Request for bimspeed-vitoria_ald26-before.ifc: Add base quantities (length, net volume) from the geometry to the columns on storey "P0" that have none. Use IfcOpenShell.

First a look at what the model holds.

```python
import ifcopenshell
import ifcopenshell.util.element
import ifcopenshell.util.unit

model = ifcopenshell.open("bimspeed-vitoria_ald26-before.ifc")
print(model.schema)
for unit_type in ("LENGTHUNIT", "AREAUNIT", "VOLUMEUNIT"):
    print(unit_type, ifcopenshell.util.unit.calculate_unit_scale(model, unit_type))
storey = next(s for s in model.by_type("IfcBuildingStorey") if s.Name == "P0")
columns = [e for e in ifcopenshell.util.element.get_decomposition(storey) if e.is_a("IfcColumn")]
for e in sorted(columns, key=lambda e: e.id()):
    print(e.id(), e.is_a(), e.Name, list(ifcopenshell.util.element.get_psets(e, qtos_only=True)), sep=" | ")
```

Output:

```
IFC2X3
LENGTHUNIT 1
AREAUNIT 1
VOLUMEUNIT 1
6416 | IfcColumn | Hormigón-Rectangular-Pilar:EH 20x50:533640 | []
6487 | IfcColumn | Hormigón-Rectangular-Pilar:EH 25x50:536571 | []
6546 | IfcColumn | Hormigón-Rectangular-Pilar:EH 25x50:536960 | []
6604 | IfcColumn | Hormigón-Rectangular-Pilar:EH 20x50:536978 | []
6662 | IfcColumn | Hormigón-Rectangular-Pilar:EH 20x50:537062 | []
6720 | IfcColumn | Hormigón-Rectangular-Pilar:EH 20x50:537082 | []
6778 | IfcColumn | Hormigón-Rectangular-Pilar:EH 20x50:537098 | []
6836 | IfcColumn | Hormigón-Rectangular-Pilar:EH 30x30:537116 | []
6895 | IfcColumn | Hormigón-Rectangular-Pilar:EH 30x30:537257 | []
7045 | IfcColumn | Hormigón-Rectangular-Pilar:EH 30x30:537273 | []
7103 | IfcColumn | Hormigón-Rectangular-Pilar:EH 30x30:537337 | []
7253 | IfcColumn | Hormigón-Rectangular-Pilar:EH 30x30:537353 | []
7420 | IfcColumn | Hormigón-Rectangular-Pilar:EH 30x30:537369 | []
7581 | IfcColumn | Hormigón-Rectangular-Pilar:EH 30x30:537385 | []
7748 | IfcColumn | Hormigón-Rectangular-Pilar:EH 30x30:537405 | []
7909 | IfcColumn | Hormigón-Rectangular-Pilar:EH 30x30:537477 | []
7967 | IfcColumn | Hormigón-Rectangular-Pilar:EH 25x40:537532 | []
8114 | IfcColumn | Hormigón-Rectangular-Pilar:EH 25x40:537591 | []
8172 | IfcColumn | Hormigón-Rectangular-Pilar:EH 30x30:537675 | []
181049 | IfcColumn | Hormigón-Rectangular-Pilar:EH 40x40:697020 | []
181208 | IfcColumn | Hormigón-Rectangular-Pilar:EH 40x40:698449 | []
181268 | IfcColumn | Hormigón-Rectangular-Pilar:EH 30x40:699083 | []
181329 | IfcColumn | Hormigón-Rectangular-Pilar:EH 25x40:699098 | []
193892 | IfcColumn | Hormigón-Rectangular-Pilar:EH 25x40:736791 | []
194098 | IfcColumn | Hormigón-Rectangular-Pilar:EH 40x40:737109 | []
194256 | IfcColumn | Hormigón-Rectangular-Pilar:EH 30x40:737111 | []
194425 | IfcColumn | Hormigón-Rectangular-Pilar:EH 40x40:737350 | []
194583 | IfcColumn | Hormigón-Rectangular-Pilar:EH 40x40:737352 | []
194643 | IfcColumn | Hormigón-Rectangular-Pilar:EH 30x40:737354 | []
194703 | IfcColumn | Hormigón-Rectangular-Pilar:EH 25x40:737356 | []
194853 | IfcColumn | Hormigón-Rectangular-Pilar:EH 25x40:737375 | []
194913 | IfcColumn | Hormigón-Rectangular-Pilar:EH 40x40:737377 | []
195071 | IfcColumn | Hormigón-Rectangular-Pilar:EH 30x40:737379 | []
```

```python
import ifcopenshell
import ifcopenshell.api.pset
import ifcopenshell.geom
import ifcopenshell.util.element
import ifcopenshell.util.shape
import ifcopenshell.util.unit

model = ifcopenshell.open("bimspeed-vitoria_ald26-before.ifc")
unit_scale = ifcopenshell.util.unit.calculate_unit_scale(model)
volume_scale = ifcopenshell.util.unit.calculate_unit_scale(model, "VOLUMEUNIT")
settings = ifcopenshell.geom.settings()

storey = next(s for s in model.by_type("IfcBuildingStorey") if s.Name == "P0")
columns = [e for e in ifcopenshell.util.element.get_decomposition(storey) if e.is_a("IfcColumn")]

for e in sorted(columns, key=lambda e: e.id()):
    if ifcopenshell.util.element.get_psets(e, qtos_only=True, should_inherit=False):
        continue
    # Geometry comes back in metres, in the element's own axes.
    shape = ifcopenshell.geom.create_shape(settings, e)
    values = {
        "Length": ifcopenshell.util.shape.get_z(shape.geometry) / unit_scale,
        "NetVolume": ifcopenshell.util.shape.get_volume(shape.geometry) / volume_scale,
    }
    qto = ifcopenshell.api.pset.add_qto(model, product=e, name="BaseQuantities")
    ifcopenshell.api.pset.edit_qto(model, qto=qto, properties=values)
    print(e.id(), {k: round(v, 3) for k, v in values.items()})

model.write("bimspeed-vitoria_ald26-before_v2.ifc")
```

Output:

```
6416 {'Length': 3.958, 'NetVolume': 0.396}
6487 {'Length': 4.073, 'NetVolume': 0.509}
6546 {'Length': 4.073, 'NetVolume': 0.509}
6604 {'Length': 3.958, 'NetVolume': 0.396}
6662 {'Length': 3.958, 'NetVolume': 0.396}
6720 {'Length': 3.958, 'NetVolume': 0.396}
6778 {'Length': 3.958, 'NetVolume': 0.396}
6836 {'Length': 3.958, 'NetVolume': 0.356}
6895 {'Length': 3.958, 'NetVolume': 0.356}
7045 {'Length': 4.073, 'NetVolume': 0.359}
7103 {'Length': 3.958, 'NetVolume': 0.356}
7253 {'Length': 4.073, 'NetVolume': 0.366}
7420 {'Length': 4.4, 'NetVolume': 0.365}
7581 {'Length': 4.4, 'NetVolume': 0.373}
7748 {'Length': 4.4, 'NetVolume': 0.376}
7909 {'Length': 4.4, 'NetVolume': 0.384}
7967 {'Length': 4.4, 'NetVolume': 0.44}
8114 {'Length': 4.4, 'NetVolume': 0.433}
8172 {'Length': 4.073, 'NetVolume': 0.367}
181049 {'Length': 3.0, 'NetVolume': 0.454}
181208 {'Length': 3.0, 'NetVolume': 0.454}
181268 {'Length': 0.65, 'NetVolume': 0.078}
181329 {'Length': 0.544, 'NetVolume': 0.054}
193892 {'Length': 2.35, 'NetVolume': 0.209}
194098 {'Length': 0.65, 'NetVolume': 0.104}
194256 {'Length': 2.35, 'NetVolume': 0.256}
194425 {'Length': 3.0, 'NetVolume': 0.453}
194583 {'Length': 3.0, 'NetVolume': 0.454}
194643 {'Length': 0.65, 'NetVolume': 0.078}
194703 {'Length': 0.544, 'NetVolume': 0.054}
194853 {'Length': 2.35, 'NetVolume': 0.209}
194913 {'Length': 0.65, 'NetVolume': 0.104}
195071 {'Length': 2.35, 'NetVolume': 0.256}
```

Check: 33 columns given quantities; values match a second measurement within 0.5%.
